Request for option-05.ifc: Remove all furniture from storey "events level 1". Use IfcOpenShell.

First a look at what the model holds.

```python
import ifcopenshell
import ifcopenshell.util.element

model = ifcopenshell.open("option-05.ifc")
print(model.schema)
storey = next(s for s in model.by_type("IfcBuildingStorey") if s.Name == "events level 1")
furniture = [e for e in ifcopenshell.util.element.get_decomposition(storey) if e.is_a("IfcFurnishingElement")]
seen = {}
for e in furniture:
    element_type = ifcopenshell.util.element.get_type(e)
    name = element_type.Name if element_type not in (None, e) else None
    seen[name] = seen.get(name, 0) + 1
for name, count in sorted(seen.items(), key=str):
    print(count, "x", name)
```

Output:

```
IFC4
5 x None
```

```python
import ifcopenshell
import ifcopenshell.api.root
import ifcopenshell.util.element

model = ifcopenshell.open("option-05.ifc")

storey = next(s for s in model.by_type("IfcBuildingStorey") if s.Name == "events level 1")
furniture = [e for e in ifcopenshell.util.element.get_decomposition(storey) if e.is_a("IfcFurnishingElement")]

for e in furniture:
    ifcopenshell.api.root.remove_product(model, product=e)
print(len(furniture), "removed")

model.write("option-05_updated.ifc")
```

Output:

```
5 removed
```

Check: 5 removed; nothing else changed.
